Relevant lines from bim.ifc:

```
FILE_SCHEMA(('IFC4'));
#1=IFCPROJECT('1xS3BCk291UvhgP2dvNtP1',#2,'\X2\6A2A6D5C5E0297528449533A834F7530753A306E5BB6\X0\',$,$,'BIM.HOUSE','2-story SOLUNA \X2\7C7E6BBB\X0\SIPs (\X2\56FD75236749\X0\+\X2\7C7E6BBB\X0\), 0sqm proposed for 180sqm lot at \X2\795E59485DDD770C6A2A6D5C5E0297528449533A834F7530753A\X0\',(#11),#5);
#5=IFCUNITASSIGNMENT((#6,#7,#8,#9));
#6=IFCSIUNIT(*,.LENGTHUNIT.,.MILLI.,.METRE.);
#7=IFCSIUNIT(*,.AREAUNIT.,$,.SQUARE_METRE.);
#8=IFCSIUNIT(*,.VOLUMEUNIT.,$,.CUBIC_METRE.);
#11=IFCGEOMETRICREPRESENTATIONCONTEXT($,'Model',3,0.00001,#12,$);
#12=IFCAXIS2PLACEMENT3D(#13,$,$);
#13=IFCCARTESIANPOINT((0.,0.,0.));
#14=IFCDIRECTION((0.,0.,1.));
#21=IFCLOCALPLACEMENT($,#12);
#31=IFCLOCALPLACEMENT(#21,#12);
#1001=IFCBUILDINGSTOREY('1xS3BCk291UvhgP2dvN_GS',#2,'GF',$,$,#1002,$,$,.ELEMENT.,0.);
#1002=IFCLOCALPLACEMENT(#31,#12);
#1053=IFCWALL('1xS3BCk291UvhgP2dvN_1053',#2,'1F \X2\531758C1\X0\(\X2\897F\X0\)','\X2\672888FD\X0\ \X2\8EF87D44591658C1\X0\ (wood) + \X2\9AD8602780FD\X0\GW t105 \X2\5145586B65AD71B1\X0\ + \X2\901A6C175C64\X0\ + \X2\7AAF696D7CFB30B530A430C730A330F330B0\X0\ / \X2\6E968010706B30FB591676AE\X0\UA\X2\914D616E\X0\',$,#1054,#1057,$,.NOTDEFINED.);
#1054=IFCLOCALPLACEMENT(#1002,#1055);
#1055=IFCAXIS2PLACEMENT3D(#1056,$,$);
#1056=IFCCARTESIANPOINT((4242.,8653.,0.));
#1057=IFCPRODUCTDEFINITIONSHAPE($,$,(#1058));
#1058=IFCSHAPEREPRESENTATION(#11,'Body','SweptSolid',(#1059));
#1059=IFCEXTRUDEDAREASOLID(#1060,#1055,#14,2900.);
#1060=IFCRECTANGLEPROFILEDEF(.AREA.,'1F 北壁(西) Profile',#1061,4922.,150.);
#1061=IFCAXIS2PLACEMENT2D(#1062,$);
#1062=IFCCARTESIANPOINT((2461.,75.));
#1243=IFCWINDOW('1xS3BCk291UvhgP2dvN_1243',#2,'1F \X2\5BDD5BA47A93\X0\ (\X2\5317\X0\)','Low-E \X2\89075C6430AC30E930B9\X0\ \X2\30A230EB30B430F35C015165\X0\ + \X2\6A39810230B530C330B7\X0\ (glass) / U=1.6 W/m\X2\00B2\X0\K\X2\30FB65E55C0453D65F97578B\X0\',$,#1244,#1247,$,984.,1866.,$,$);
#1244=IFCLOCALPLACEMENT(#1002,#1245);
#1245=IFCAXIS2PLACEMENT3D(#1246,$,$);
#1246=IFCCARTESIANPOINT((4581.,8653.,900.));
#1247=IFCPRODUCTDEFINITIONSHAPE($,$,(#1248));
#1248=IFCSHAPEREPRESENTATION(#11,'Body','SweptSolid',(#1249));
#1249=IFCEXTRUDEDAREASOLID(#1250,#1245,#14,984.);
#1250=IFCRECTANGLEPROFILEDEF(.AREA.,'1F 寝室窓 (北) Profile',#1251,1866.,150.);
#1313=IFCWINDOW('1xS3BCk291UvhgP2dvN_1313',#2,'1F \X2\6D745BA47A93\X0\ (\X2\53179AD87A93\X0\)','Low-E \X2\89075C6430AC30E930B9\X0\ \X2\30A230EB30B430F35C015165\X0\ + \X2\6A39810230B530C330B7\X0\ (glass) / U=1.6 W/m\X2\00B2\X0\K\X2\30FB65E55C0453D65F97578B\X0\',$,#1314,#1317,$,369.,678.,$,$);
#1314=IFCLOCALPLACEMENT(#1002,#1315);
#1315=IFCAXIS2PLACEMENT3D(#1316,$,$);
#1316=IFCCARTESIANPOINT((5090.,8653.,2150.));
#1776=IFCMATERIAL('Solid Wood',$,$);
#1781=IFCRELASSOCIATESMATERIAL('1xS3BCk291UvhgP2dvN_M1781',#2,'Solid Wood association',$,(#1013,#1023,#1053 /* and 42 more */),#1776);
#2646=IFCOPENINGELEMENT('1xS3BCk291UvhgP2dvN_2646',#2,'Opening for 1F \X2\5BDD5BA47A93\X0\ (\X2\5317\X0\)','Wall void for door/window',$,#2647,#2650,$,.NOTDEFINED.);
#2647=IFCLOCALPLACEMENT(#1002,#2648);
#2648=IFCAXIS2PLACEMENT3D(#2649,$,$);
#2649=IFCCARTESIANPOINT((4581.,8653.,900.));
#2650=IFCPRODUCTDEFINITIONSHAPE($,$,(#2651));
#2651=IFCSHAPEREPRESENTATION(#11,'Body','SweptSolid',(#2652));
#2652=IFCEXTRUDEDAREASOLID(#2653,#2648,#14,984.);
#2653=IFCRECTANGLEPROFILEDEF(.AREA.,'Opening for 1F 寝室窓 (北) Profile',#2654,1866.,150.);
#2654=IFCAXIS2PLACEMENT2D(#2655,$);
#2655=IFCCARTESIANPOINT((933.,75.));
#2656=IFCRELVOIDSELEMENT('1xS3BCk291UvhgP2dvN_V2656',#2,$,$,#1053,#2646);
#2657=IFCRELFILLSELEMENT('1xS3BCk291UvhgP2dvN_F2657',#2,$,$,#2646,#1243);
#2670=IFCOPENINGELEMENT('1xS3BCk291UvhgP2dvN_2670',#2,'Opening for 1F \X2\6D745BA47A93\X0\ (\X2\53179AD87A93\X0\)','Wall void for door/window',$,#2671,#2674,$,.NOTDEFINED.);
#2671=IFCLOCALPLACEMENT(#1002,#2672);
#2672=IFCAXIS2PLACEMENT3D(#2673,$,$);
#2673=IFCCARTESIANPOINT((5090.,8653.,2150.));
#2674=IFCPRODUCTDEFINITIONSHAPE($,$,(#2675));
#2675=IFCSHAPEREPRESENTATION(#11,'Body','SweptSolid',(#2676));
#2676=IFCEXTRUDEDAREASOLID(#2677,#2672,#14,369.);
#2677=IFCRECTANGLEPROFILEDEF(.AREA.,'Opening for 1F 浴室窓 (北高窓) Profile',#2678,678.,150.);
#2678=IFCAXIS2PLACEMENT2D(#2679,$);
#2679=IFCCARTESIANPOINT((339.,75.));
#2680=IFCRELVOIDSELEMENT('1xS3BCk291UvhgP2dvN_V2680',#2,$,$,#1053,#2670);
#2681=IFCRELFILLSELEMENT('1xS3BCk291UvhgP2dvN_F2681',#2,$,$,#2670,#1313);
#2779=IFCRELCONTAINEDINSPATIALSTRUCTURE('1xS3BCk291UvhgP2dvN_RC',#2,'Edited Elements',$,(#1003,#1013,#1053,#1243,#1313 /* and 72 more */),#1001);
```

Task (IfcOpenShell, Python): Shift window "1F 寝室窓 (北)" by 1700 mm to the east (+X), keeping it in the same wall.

```python
import ifcopenshell
import ifcopenshell.api.geometry
import ifcopenshell.util.placement

model = ifcopenshell.open("bim.ifc")

window = model.by_guid("1xS3BCk291UvhgP2dvN_1243")
opening = window.FillsVoids[0].RelatingOpeningElement
wall = opening.VoidsElements[0].RelatingBuildingElement

wall_matrix = ifcopenshell.util.placement.get_local_placement(wall.ObjectPlacement)
shift = wall_matrix[:3, 0] * 1700.0
before = ifcopenshell.util.placement.get_local_placement(window.ObjectPlacement)[:3, 3].copy()

# The window is not placed relative to its opening, so move both.
for product in (opening, window):
    matrix = ifcopenshell.util.placement.get_local_placement(product.ObjectPlacement)
    matrix[:3, 3] += shift
    ifcopenshell.api.geometry.edit_object_placement(model, product=product, matrix=matrix, is_si=False)

after = ifcopenshell.util.placement.get_local_placement(window.ObjectPlacement)[:3, 3]
print("window moved by", (after - before).round(3) + 0.0)

model.write("bim_rev.ifc")
```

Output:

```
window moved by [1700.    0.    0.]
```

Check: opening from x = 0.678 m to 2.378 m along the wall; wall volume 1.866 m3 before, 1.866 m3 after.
